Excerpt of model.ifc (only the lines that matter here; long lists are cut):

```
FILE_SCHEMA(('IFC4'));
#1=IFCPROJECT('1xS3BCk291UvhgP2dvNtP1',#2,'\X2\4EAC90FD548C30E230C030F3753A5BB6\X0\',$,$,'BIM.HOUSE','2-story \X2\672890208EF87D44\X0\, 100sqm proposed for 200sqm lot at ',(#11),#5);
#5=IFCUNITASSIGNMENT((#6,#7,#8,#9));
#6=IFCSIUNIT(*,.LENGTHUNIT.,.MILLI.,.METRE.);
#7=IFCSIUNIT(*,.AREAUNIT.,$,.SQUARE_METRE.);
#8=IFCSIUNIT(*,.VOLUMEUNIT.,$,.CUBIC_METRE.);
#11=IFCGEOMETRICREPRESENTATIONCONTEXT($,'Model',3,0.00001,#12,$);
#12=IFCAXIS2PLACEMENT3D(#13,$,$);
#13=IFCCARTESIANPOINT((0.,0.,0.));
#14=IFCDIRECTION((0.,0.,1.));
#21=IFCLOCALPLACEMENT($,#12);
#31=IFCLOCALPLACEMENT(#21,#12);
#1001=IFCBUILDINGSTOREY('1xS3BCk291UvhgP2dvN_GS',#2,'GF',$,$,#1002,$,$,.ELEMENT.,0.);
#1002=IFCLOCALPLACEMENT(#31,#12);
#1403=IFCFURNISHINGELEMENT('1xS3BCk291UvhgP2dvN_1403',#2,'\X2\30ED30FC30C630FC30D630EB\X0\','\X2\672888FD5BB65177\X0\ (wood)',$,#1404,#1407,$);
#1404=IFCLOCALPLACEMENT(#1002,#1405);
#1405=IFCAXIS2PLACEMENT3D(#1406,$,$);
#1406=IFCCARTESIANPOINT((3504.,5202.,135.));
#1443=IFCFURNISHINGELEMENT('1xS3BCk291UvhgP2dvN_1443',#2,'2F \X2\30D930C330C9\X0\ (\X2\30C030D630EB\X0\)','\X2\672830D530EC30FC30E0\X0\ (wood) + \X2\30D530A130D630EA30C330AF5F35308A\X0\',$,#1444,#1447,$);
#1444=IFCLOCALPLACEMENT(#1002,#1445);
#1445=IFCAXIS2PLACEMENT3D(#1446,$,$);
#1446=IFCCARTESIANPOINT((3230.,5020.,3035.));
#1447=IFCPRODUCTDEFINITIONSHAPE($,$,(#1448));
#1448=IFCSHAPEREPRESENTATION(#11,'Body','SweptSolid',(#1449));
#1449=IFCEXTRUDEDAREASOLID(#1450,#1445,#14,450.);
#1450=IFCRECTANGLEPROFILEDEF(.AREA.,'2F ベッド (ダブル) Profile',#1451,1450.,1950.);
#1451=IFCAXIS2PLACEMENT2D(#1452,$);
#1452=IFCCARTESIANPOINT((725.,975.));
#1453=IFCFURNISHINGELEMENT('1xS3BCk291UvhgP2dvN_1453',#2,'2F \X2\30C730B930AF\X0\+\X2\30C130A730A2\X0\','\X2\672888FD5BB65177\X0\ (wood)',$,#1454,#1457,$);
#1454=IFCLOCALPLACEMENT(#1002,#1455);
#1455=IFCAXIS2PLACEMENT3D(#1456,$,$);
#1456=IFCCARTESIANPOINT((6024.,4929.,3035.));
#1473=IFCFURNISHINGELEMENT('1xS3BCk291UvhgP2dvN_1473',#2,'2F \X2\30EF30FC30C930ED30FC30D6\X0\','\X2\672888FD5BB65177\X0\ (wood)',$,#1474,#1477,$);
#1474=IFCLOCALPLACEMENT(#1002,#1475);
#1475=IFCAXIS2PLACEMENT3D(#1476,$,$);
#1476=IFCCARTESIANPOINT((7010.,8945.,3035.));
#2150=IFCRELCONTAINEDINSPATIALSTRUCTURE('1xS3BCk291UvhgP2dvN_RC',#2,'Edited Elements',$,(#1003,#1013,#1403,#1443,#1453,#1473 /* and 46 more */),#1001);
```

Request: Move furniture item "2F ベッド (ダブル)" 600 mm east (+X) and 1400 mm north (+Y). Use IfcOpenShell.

```python
import ifcopenshell
import ifcopenshell.api.geometry
import ifcopenshell.util.placement
import ifcopenshell.util.unit

model = ifcopenshell.open("model.ifc")
unit_scale = ifcopenshell.util.unit.calculate_unit_scale(model)

item = model.by_guid("1xS3BCk291UvhgP2dvN_1443")
matrix = ifcopenshell.util.placement.get_local_placement(item.ObjectPlacement)
matrix[0, 3] += 0.6 / unit_scale
matrix[1, 3] += 1.4 / unit_scale
ifcopenshell.api.geometry.edit_object_placement(model, product=item, matrix=matrix, is_si=False)

print(ifcopenshell.util.placement.get_local_placement(item.ObjectPlacement).round(3) + 0.0)

model.write("model_v2.ifc")
```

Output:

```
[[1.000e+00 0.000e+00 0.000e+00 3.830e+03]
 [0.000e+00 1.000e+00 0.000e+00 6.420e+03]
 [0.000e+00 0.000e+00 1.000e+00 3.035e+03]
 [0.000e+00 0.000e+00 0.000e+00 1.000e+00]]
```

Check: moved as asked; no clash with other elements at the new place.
